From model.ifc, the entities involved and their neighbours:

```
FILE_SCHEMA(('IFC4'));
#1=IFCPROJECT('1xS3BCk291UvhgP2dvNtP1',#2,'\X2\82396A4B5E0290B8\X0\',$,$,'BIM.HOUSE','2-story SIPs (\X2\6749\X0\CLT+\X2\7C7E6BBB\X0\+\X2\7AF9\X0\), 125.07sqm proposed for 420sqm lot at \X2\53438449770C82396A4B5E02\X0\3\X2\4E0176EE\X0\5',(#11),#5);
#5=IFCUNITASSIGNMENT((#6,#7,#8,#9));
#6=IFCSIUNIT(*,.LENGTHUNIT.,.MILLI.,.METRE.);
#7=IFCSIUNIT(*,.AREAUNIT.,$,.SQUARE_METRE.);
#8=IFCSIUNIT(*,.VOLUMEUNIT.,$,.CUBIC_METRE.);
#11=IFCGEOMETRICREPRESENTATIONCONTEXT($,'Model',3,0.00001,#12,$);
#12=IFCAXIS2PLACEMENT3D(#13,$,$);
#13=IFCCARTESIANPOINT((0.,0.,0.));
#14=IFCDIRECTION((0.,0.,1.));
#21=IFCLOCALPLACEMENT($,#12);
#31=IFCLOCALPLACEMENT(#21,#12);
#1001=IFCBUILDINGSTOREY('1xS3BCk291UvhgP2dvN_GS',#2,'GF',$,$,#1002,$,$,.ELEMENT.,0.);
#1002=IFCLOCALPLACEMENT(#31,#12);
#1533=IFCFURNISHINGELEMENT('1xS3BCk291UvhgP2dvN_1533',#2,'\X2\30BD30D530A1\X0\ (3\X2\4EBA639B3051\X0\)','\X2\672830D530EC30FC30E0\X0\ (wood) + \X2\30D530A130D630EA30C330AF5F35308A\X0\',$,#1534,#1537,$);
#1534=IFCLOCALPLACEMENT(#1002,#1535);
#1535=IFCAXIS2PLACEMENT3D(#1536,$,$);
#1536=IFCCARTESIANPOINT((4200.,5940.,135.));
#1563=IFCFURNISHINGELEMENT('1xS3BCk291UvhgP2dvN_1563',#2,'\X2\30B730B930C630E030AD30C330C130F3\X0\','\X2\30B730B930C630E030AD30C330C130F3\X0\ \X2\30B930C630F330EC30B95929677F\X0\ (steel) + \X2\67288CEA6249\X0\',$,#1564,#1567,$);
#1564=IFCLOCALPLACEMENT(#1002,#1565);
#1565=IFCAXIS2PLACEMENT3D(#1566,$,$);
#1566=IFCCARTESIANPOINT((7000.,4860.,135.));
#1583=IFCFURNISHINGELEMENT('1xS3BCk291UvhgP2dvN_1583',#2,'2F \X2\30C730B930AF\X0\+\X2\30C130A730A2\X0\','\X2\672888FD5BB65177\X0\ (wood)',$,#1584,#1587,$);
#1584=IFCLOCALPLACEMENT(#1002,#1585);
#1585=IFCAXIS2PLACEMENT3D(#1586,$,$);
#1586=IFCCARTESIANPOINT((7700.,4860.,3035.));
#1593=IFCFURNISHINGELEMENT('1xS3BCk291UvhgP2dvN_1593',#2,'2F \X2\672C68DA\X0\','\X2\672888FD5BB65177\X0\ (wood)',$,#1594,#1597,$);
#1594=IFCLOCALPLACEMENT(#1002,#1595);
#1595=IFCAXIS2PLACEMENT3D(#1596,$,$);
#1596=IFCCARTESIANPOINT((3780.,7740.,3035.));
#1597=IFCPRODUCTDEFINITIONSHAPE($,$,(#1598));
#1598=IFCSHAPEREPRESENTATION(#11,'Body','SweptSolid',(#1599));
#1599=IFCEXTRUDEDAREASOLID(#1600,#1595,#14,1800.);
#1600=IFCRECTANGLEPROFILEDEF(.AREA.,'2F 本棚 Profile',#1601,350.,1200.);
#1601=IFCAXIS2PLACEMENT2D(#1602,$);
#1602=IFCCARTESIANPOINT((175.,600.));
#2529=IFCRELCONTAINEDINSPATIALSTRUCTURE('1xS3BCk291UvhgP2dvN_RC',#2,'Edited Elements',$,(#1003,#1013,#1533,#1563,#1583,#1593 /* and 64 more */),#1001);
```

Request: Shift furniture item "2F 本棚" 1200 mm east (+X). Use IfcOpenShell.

```python
import ifcopenshell
import ifcopenshell.api.geometry
import ifcopenshell.util.placement
import ifcopenshell.util.unit

model = ifcopenshell.open("model.ifc")
unit_scale = ifcopenshell.util.unit.calculate_unit_scale(model)

item = model.by_guid("1xS3BCk291UvhgP2dvN_1593")
matrix = ifcopenshell.util.placement.get_local_placement(item.ObjectPlacement)
matrix[0, 3] += 1.2 / unit_scale
ifcopenshell.api.geometry.edit_object_placement(model, product=item, matrix=matrix, is_si=False)

print(ifcopenshell.util.placement.get_local_placement(item.ObjectPlacement).round(3) + 0.0)

model.write("model_v2.ifc")
```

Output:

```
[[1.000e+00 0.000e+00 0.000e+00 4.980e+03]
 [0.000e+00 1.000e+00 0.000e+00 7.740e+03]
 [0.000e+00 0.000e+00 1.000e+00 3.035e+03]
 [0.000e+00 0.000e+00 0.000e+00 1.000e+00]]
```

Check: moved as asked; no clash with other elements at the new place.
